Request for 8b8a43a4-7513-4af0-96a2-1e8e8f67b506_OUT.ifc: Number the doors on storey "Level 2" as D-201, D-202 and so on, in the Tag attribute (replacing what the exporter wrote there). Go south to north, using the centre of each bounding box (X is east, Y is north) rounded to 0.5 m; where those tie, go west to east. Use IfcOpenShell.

First a look at what the model holds.

```python
import ifcopenshell
import ifcopenshell.util.element
import ifcopenshell.util.placement

model = ifcopenshell.open("8b8a43a4-7513-4af0-96a2-1e8e8f67b506_OUT.ifc")
print(model.schema)
storey = next(s for s in model.by_type("IfcBuildingStorey") if s.Name == "Level 2")
doors = [e for e in ifcopenshell.util.element.get_decomposition(storey) if e.is_a("IfcDoor")]
for e in sorted(doors, key=lambda e: e.id()):
    origin = ifcopenshell.util.placement.get_local_placement(e.ObjectPlacement)[:3, 3]
    print(e.id(), e.Tag, e.Name, origin.round(2) + 0.0, sep=" | ")
```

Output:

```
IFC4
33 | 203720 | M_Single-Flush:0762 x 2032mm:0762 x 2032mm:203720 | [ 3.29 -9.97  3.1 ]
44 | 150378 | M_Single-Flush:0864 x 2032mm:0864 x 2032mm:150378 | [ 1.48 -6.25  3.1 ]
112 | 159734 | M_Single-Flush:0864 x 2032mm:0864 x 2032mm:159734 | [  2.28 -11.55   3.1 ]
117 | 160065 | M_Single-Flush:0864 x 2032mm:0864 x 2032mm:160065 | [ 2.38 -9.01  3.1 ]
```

```python
import ifcopenshell
import ifcopenshell.geom
import ifcopenshell.util.element
import ifcopenshell.util.shape

model = ifcopenshell.open("8b8a43a4-7513-4af0-96a2-1e8e8f67b506_OUT.ifc")
settings = ifcopenshell.geom.settings()
settings.set("use-world-coords", True)


def centre(element):
    shape = ifcopenshell.geom.create_shape(settings, element)
    return ifcopenshell.util.shape.get_bbox_centroid(shape.geometry)


storey = next(s for s in model.by_type("IfcBuildingStorey") if s.Name == "Level 2")
doors = [e for e in ifcopenshell.util.element.get_decomposition(storey) if e.is_a("IfcDoor")]

# Insertion points can sit at a corner or the storey origin, so sort by the geometry (in metres).
centres = {e: centre(e) for e in doors}
doors.sort(key=lambda e: (round(centres[e][1] / 0.5), centres[e][0]))

for i, e in enumerate(doors, start=1):
    number = f"D-2{i:02d}"
    e.Tag = number
    print(e.id(), number)

model.write("8b8a43a4-7513-4af0-96a2-1e8e8f67b506_OUT_v2.ifc")
```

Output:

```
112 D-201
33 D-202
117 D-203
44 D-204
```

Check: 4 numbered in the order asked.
